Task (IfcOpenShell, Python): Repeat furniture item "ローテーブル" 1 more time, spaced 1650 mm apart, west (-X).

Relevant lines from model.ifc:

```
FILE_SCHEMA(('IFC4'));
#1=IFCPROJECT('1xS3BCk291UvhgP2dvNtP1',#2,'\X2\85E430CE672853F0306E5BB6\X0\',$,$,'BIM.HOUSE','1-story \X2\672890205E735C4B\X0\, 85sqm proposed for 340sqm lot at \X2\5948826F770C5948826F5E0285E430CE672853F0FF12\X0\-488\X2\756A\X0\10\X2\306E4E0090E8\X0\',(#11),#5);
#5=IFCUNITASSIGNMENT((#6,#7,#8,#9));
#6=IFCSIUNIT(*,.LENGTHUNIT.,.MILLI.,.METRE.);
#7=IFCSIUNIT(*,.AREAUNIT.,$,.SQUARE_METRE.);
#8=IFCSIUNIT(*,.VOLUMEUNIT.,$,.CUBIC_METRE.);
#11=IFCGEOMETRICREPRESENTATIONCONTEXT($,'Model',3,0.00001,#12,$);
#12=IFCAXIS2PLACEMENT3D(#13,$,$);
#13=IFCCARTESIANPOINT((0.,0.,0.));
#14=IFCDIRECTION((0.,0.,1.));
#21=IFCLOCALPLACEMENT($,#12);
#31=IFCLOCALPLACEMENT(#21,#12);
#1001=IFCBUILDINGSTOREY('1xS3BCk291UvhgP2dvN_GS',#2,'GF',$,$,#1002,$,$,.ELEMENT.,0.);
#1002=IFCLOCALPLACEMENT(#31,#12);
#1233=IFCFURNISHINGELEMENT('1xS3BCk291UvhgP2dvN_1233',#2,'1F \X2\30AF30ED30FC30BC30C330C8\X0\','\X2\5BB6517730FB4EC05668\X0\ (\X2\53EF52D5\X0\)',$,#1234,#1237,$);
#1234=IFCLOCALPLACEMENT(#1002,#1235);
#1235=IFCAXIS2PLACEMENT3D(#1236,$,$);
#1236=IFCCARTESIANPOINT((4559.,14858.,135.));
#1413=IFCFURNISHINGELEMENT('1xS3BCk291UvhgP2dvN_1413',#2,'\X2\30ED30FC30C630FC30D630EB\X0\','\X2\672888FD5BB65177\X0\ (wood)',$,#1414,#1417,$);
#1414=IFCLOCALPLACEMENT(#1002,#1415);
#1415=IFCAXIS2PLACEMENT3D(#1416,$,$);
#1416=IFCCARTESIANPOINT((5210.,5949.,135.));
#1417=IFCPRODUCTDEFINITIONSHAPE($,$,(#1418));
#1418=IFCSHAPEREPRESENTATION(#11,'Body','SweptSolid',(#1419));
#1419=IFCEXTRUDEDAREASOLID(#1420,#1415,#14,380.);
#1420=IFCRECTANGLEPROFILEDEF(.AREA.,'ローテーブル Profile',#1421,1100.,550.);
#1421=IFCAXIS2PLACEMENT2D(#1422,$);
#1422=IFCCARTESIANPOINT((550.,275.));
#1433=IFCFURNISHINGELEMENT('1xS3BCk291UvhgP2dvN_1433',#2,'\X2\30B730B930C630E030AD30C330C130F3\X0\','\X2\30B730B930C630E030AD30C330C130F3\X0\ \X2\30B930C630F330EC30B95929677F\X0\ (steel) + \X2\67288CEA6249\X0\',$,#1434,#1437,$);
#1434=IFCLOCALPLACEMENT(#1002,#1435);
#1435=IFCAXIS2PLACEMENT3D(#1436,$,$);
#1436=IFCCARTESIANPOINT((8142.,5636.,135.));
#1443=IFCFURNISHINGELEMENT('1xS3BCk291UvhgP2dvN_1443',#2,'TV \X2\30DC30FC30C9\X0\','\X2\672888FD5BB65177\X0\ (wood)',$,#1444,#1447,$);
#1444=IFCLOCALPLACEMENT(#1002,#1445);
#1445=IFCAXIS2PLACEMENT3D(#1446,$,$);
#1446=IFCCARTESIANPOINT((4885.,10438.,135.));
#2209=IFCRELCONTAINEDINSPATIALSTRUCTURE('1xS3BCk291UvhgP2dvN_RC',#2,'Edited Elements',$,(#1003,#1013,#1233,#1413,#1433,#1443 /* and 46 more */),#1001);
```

```python
import numpy as np
import ifcopenshell
import ifcopenshell.api.geometry
import ifcopenshell.api.root
import ifcopenshell.util.element
import ifcopenshell.util.placement
import ifcopenshell.util.unit

model = ifcopenshell.open("model.ifc")
unit_scale = ifcopenshell.util.unit.calculate_unit_scale(model)


def reuse_history(source, copy):
    """copy_class also copies each property set's owner history, people and application; keep the originals."""
    for rel in copy.IsDefinedBy:
        if rel.is_a("IfcRelDefinesByProperties") and (history := rel.RelatingPropertyDefinition.OwnerHistory):
            rel.RelatingPropertyDefinition.OwnerHistory = source.OwnerHistory
            ifcopenshell.util.element.remove_deep2(model, history)


source = model.by_id(1413)
base = ifcopenshell.util.placement.get_local_placement(source.ObjectPlacement)
step = np.array([-1.0, 0.0, 0.0]) * 1.65 / unit_scale

for i in range(1, 2):
    copy = ifcopenshell.api.root.copy_class(model, product=source)
    copy.Representation = ifcopenshell.util.element.copy_deep(
        model, source.Representation, exclude=["IfcGeometricRepresentationContext", "IfcRepresentationMap"]
    )
    reuse_history(source, copy)
    matrix = base.copy()
    matrix[:3, 3] += i * step
    print("added at", matrix[:3, 3].round(3) + 0.0)
    ifcopenshell.api.geometry.edit_object_placement(model, product=copy, matrix=matrix, is_si=False)

model.write("model_updated.ifc")
```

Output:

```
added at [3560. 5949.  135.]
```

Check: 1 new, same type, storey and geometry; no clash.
